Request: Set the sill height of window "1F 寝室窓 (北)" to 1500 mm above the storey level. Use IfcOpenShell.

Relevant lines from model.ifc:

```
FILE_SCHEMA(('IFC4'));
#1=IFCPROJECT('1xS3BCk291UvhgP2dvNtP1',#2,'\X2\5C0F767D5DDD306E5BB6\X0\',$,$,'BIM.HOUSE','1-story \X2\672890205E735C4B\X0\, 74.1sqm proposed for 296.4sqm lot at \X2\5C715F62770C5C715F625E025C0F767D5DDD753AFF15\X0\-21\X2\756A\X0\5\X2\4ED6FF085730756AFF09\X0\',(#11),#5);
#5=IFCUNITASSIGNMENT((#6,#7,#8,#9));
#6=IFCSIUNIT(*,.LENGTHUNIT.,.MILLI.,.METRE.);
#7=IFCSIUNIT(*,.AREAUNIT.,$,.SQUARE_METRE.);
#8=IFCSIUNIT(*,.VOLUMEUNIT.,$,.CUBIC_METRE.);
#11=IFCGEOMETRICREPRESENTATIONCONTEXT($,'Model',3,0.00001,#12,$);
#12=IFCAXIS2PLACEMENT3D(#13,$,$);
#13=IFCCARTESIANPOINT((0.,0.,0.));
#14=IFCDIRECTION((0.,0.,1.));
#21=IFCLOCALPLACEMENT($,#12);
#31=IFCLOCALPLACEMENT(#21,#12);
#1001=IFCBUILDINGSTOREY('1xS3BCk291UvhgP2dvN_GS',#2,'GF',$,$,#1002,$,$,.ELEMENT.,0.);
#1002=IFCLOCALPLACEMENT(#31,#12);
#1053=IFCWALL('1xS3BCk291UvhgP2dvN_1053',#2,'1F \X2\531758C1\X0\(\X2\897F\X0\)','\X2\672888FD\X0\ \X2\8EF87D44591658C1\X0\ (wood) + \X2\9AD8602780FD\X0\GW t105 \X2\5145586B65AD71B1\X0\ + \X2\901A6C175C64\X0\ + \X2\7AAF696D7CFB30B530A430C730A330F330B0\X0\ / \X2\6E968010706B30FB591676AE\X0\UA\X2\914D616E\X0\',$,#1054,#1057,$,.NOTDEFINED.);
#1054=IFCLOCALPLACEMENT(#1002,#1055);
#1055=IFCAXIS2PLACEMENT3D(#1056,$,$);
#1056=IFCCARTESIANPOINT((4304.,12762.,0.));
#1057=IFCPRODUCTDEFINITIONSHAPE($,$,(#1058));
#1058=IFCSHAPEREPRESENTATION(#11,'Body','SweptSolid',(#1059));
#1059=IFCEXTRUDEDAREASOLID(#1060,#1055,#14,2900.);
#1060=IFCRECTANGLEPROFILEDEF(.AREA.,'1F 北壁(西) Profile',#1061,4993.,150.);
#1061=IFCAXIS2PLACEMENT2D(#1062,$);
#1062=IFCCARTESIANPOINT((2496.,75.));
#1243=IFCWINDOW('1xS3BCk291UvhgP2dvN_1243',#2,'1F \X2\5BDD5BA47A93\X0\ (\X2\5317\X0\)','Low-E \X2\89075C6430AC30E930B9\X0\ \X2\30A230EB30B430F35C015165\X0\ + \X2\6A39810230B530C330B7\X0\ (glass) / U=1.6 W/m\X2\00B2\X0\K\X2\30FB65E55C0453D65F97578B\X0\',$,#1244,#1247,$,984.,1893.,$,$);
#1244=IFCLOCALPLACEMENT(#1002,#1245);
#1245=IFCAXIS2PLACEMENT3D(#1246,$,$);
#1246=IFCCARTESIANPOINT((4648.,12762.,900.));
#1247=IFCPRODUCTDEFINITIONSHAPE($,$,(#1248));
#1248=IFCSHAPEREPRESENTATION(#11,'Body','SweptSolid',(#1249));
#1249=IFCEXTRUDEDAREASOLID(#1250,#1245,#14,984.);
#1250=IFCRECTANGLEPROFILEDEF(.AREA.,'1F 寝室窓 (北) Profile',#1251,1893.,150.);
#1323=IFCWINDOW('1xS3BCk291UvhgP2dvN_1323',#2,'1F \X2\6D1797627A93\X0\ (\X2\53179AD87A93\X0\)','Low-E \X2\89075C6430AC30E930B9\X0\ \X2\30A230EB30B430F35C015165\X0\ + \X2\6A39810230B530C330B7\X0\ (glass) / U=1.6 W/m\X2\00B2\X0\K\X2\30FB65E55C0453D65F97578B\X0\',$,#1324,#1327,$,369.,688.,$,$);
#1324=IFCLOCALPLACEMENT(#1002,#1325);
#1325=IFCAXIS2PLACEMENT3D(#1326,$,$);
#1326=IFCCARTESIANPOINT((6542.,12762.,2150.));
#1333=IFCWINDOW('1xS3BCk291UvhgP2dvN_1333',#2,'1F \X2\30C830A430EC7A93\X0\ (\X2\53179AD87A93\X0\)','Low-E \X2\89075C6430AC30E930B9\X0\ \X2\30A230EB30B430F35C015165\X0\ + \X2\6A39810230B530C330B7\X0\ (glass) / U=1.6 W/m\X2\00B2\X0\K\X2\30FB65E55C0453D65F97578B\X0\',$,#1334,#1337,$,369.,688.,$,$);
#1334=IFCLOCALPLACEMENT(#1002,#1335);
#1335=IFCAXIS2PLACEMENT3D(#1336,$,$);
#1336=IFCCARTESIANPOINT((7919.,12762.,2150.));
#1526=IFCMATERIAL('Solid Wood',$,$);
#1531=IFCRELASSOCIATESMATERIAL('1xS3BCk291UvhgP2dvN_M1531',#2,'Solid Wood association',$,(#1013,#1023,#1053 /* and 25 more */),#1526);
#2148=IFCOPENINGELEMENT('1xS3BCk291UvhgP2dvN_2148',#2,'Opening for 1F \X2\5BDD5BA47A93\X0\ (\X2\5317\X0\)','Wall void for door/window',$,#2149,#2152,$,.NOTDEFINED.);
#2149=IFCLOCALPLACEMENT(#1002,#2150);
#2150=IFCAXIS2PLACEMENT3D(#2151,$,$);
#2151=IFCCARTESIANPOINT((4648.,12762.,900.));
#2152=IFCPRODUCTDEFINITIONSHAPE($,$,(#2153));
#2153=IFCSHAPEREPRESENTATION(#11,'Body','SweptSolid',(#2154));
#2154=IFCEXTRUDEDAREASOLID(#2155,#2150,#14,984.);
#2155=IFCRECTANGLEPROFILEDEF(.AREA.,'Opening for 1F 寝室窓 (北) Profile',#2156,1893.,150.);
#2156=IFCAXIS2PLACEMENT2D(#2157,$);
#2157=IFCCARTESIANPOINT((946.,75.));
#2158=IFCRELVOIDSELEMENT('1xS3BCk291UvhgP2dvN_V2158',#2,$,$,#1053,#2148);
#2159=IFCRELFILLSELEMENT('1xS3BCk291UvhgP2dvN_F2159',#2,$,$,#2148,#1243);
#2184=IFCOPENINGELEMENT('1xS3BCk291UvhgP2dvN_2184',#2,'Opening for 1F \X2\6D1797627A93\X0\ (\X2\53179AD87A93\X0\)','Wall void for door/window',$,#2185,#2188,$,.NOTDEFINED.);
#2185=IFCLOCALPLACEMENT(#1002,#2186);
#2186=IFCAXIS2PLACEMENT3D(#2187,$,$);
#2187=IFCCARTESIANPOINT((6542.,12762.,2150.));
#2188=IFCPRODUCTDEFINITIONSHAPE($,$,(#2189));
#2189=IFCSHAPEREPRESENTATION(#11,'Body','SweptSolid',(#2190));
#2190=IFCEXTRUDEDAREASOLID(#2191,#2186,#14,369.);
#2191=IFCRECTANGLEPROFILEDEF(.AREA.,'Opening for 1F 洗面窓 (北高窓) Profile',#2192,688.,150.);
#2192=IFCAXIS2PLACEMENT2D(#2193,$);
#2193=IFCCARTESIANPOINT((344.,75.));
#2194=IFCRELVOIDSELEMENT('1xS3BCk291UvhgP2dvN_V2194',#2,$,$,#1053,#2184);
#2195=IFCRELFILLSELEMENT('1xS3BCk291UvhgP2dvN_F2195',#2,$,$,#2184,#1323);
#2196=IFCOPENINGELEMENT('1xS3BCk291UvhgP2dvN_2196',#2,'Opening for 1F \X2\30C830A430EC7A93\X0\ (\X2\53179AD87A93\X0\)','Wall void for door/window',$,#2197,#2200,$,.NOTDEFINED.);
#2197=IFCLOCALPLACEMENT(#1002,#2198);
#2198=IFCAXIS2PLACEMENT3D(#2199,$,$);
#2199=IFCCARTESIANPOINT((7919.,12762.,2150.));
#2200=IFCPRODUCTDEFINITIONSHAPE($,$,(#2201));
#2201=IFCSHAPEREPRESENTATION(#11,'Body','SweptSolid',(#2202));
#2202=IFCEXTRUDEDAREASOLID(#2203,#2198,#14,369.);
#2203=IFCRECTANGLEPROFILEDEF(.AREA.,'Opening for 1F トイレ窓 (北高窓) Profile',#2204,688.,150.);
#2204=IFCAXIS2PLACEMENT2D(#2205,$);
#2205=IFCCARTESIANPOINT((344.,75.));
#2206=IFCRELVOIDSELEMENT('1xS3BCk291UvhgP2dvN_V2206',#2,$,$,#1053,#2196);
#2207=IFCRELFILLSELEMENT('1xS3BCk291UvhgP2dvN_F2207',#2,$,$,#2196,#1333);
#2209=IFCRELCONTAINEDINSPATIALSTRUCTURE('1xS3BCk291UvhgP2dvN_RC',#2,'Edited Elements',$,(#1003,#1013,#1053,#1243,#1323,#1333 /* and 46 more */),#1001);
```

```python
import numpy as np
import ifcopenshell
import ifcopenshell.api.geometry
import ifcopenshell.geom
import ifcopenshell.util.element
import ifcopenshell.util.placement
import ifcopenshell.util.shape
import ifcopenshell.util.unit

model = ifcopenshell.open("model.ifc")
unit_scale = ifcopenshell.util.unit.calculate_unit_scale(model)

window = model.by_guid("1xS3BCk291UvhgP2dvN_1243")
opening = window.FillsVoids[0].RelatingOpeningElement
storey = ifcopenshell.util.element.get_container(window, ifc_class="IfcBuildingStorey")
level = ifcopenshell.util.placement.get_local_placement(storey.ObjectPlacement)[2, 3]

# The opening's origin need not be at the sill, so measure its lowest point.
shape = ifcopenshell.geom.create_shape(ifcopenshell.geom.settings(), opening)
bottom = ifcopenshell.util.shape.get_shape_bottom_elevation(shape, shape.geometry) / unit_scale
dz = level + 1.5 / unit_scale - bottom

shift = np.array([0.0, 0.0, dz])
# The window is not placed relative to its opening, so move both.
for product in (opening, window):
    matrix = ifcopenshell.util.placement.get_local_placement(product.ObjectPlacement)
    matrix[:3, 3] += shift
    ifcopenshell.api.geometry.edit_object_placement(model, product=product, matrix=matrix, is_si=False)

print(f"moved by {dz * unit_scale:+.3f} m")

model.write("model_rev.ifc")
```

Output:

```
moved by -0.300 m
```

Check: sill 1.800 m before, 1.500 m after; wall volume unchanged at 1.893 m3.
